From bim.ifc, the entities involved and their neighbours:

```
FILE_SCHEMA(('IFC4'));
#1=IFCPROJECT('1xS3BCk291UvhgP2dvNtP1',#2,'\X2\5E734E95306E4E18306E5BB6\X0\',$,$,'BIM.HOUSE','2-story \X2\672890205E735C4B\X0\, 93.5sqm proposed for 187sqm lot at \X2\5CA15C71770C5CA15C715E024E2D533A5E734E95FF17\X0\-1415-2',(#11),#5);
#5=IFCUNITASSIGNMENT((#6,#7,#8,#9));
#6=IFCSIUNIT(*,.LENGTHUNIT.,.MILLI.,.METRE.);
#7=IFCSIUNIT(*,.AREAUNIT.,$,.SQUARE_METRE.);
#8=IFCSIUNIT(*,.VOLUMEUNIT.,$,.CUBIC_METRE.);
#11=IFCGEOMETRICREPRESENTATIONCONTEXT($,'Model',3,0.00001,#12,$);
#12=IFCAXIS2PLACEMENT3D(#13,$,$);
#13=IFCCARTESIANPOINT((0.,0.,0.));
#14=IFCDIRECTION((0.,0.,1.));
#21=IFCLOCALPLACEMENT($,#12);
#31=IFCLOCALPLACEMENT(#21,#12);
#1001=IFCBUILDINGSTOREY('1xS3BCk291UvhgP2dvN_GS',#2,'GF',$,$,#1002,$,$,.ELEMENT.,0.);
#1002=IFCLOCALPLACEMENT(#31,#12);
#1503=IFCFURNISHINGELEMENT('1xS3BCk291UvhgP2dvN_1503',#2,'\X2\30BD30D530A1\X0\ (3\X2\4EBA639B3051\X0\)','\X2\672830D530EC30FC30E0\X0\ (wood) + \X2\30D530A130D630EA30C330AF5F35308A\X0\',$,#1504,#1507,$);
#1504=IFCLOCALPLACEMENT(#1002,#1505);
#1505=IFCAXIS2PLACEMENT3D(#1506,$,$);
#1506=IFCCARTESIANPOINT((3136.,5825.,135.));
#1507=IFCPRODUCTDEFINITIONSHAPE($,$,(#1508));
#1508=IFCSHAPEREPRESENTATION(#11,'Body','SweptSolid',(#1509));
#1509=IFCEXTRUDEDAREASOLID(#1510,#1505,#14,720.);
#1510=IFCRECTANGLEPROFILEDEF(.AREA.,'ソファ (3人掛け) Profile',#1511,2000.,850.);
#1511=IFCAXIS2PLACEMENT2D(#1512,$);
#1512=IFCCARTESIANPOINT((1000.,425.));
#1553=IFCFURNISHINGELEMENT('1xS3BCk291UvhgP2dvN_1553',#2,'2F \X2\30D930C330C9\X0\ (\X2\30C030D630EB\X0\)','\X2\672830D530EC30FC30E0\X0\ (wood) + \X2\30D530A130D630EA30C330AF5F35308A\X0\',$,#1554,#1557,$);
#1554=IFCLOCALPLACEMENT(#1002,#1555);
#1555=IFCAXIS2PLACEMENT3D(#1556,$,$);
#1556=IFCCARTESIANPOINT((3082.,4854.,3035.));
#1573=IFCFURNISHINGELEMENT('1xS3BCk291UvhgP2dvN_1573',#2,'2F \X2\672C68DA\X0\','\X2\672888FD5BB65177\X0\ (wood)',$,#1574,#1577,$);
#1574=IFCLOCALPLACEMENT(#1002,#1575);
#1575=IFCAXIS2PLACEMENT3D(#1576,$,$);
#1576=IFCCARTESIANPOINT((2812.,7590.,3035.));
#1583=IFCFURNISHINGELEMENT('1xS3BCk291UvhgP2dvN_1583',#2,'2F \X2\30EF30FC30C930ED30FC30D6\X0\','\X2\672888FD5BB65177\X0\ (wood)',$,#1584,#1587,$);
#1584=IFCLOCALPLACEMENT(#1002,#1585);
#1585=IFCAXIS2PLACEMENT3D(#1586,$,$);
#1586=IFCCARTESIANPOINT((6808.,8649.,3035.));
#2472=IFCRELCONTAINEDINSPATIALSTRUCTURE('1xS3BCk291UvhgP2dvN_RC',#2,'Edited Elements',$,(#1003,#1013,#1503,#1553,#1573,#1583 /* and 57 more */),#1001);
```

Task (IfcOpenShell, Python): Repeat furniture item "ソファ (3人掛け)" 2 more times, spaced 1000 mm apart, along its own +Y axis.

```python
import ifcopenshell
import ifcopenshell.api.geometry
import ifcopenshell.api.root
import ifcopenshell.util.element
import ifcopenshell.util.placement

model = ifcopenshell.open("bim.ifc")


def reuse_history(source, copy):
    """copy_class also copies each property set's owner history, people and application; keep the originals."""
    for rel in copy.IsDefinedBy:
        if rel.is_a("IfcRelDefinesByProperties") and (history := rel.RelatingPropertyDefinition.OwnerHistory):
            rel.RelatingPropertyDefinition.OwnerHistory = source.OwnerHistory
            ifcopenshell.util.element.remove_deep2(model, history)


source = model.by_guid("1xS3BCk291UvhgP2dvN_1503")
base = ifcopenshell.util.placement.get_local_placement(source.ObjectPlacement)
step = base[:3, 1] * 1000.0

for i in range(1, 3):
    copy = ifcopenshell.api.root.copy_class(model, product=source)
    copy.Representation = ifcopenshell.util.element.copy_deep(
        model, source.Representation, exclude=["IfcGeometricRepresentationContext", "IfcRepresentationMap"]
    )
    reuse_history(source, copy)
    matrix = base.copy()
    matrix[:3, 3] += i * step
    print("added at", matrix[:3, 3].round(3) + 0.0)
    ifcopenshell.api.geometry.edit_object_placement(model, product=copy, matrix=matrix, is_si=False)

model.write("bim_v2.ifc")
```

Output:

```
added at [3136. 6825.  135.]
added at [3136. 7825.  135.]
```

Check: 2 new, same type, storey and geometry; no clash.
